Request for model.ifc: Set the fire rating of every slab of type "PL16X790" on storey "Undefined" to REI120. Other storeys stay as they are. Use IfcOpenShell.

First a look at what the model holds.

```python
import ifcopenshell
import ifcopenshell.util.element

model = ifcopenshell.open("model.ifc")
print(model.schema)
storey = next(s for s in model.by_type("IfcBuildingStorey") if s.Name == "Undefined")
slabs = [e for e in ifcopenshell.util.element.get_decomposition(storey) if e.is_a("IfcSlab")]
seen = {}
for e in slabs:
    element_type = ifcopenshell.util.element.get_type(e)
    key = (element_type.Name if element_type != e and element_type else None, ifcopenshell.util.element.get_pset(e, "Pset_SlabCommon", "FireRating"))
    seen[key] = seen.get(key, 0) + 1
for (name, value), count in sorted(seen.items(), key=str):
    print(count, "x", name, "|", value)
```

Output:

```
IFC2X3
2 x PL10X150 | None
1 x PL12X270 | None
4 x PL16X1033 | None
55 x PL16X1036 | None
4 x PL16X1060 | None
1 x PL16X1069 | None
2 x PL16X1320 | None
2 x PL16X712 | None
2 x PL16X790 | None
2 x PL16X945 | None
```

```python
import ifcopenshell
import ifcopenshell.api.pset
import ifcopenshell.util.element

model = ifcopenshell.open("model.ifc")

storey = next(s for s in model.by_type("IfcBuildingStorey") if s.Name == "Undefined")
slabs = [e for e in ifcopenshell.util.element.get_decomposition(storey) if e.is_a("IfcSlab")]

count = 0
for e in slabs:
    element_type = ifcopenshell.util.element.get_type(e)
    if element_type in (None, e) or element_type.Name != "PL16X790":
        continue
    # add_pset returns the element's existing set when there is one.
    pset = ifcopenshell.api.pset.add_pset(model, product=e, name="Pset_SlabCommon")
    ifcopenshell.api.pset.edit_pset(model, pset=pset, properties={"FireRating": "REI120"})
    count += 1

print(count, "slabs updated")

model.write("model-out.ifc")
```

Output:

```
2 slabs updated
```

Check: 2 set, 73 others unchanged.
